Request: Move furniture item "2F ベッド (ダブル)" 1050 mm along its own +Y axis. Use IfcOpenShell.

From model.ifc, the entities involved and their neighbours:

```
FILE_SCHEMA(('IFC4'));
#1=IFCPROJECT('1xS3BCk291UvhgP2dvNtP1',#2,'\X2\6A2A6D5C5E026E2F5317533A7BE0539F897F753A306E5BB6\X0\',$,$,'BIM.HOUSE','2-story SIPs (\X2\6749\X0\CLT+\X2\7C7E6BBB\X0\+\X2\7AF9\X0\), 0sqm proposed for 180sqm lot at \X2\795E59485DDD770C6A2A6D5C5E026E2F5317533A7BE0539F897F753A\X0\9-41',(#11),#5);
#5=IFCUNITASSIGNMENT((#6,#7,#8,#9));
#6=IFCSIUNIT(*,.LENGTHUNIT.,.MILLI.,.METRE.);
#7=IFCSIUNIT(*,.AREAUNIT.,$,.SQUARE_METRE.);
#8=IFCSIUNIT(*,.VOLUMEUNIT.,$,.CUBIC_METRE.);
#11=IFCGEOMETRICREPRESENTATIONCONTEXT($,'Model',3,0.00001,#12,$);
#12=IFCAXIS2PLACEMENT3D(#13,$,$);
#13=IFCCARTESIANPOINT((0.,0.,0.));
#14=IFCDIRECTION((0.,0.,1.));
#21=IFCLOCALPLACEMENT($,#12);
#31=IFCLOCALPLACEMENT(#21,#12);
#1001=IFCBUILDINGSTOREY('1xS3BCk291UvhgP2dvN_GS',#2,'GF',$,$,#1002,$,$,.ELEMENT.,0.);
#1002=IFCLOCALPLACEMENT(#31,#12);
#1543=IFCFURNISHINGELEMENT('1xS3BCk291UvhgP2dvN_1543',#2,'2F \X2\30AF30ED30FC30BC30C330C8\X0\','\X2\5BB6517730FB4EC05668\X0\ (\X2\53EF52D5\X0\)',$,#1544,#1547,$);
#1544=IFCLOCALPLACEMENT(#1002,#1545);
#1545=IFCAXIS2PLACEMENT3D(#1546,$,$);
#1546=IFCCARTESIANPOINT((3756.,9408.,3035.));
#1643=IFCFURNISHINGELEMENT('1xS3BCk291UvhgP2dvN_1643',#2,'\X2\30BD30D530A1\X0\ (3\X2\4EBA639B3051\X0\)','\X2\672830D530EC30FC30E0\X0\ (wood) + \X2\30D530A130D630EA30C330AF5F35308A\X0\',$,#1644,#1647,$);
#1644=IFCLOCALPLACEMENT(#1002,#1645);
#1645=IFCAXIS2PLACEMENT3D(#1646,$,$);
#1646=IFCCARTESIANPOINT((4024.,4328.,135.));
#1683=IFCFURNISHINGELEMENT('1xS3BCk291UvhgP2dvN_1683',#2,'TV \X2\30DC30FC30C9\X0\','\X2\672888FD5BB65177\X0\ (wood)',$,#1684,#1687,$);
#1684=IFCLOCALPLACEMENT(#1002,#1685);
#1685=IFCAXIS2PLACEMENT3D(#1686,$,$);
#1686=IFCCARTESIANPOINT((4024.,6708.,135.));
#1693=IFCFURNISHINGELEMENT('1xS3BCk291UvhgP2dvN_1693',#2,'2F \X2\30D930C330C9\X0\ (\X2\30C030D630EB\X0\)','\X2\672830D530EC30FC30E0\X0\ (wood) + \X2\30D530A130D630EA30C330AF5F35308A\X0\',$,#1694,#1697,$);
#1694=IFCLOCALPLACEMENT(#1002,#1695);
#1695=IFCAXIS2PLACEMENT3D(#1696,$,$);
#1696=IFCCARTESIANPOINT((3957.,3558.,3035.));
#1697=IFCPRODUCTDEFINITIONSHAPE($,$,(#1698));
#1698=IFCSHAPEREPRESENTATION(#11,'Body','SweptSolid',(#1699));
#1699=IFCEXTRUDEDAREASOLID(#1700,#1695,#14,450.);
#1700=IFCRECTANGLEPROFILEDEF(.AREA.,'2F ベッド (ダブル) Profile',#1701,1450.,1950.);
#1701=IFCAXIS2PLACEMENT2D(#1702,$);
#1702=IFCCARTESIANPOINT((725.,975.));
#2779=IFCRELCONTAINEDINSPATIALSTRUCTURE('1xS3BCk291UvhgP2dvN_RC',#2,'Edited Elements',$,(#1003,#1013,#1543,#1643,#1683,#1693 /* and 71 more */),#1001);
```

```python
import ifcopenshell
import ifcopenshell.api.geometry
import ifcopenshell.util.placement
import ifcopenshell.util.unit

model = ifcopenshell.open("model.ifc")
unit_scale = ifcopenshell.util.unit.calculate_unit_scale(model)

item = model.by_id(1693)
matrix = ifcopenshell.util.placement.get_local_placement(item.ObjectPlacement)
matrix[:3, 3] += matrix[:3, 1] * 1.05 / unit_scale
ifcopenshell.api.geometry.edit_object_placement(model, product=item, matrix=matrix, is_si=False)

print(ifcopenshell.util.placement.get_local_placement(item.ObjectPlacement).round(3) + 0.0)

model.write("model-out.ifc")
```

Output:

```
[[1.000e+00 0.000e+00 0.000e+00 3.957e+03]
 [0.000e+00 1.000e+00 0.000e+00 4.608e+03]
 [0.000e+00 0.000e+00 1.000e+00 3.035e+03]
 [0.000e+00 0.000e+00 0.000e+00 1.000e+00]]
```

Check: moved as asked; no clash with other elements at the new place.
